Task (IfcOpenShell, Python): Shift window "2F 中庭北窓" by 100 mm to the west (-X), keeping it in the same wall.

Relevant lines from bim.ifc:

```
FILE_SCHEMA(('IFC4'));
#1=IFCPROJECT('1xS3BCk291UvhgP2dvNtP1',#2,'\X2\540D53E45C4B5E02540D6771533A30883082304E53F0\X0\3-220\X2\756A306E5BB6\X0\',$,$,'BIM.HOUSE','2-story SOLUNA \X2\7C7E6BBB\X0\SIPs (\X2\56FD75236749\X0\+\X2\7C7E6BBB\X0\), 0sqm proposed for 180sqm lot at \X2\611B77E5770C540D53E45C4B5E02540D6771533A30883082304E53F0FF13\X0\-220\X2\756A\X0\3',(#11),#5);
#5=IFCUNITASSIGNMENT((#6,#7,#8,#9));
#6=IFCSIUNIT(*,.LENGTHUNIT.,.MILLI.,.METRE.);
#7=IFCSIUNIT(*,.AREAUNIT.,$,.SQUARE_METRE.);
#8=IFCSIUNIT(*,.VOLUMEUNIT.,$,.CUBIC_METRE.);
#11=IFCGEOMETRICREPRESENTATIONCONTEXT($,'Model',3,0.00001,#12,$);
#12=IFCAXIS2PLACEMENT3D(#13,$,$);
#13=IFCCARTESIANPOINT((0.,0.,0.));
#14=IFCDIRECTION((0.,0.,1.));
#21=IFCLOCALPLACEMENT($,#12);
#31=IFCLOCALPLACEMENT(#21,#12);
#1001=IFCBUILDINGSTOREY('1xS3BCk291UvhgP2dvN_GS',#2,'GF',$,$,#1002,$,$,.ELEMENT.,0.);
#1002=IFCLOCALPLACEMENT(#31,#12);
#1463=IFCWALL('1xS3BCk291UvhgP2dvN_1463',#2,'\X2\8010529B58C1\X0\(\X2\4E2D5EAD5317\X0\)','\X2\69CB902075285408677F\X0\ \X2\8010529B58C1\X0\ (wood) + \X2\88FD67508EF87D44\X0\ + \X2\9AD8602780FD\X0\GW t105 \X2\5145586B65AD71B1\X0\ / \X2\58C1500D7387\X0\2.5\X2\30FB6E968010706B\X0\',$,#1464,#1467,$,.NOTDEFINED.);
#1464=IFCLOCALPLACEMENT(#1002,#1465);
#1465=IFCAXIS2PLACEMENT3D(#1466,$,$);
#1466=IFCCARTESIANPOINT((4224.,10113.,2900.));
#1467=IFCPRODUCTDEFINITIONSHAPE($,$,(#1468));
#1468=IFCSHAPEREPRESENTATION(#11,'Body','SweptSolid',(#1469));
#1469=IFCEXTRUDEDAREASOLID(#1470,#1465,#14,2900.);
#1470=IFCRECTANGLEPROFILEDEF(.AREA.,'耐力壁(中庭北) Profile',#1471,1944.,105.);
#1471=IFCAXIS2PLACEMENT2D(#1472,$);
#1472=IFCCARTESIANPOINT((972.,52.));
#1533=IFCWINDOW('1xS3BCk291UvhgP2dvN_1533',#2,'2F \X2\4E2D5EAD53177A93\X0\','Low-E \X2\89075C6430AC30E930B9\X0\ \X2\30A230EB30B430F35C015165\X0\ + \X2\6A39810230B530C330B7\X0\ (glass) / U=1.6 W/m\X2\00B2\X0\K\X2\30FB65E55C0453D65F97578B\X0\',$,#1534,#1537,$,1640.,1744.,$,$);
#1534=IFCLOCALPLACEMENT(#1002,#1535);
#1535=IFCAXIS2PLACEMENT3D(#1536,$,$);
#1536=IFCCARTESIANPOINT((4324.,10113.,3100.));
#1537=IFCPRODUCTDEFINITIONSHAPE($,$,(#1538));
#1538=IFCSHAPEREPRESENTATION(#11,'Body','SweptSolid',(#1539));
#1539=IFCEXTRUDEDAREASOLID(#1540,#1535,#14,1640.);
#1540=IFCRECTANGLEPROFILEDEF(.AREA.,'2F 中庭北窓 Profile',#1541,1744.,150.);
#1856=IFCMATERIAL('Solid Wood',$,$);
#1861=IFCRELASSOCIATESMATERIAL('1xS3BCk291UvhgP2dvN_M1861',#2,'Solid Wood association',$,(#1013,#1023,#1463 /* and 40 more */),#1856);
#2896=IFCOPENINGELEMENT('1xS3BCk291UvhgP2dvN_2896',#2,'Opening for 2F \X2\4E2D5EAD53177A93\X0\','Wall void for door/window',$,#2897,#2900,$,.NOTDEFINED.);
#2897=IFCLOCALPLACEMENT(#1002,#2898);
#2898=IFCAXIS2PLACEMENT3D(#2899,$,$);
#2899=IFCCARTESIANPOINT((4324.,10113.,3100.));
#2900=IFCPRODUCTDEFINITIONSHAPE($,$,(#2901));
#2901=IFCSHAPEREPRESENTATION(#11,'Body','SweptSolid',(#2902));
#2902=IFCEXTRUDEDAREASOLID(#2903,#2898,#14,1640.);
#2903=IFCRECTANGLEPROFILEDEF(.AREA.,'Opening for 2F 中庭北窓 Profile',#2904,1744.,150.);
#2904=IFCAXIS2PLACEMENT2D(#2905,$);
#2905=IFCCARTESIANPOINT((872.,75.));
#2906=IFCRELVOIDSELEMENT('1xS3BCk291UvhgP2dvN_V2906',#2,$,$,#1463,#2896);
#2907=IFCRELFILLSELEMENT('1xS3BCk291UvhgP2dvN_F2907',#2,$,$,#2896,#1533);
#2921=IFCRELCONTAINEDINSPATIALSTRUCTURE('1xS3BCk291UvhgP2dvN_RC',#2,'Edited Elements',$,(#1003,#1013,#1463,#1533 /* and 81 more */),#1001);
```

```python
import ifcopenshell
import ifcopenshell.api.geometry
import ifcopenshell.util.placement
import ifcopenshell.util.unit

model = ifcopenshell.open("bim.ifc")
unit_scale = ifcopenshell.util.unit.calculate_unit_scale(model)

window = model.by_guid("1xS3BCk291UvhgP2dvN_1533")
opening = window.FillsVoids[0].RelatingOpeningElement
wall = opening.VoidsElements[0].RelatingBuildingElement

wall_matrix = ifcopenshell.util.placement.get_local_placement(wall.ObjectPlacement)
shift = wall_matrix[:3, 0] * -0.1 / unit_scale
before = ifcopenshell.util.placement.get_local_placement(window.ObjectPlacement)[:3, 3].copy()

# The window is not placed relative to its opening, so move both.
for product in (opening, window):
    matrix = ifcopenshell.util.placement.get_local_placement(product.ObjectPlacement)
    matrix[:3, 3] += shift
    ifcopenshell.api.geometry.edit_object_placement(model, product=product, matrix=matrix, is_si=False)

after = ifcopenshell.util.placement.get_local_placement(window.ObjectPlacement)[:3, 3]
print("window moved by", (after - before).round(3) + 0.0)

model.write("bim_edited.ifc")
```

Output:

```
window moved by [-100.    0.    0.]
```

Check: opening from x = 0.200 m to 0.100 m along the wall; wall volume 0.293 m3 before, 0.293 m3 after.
